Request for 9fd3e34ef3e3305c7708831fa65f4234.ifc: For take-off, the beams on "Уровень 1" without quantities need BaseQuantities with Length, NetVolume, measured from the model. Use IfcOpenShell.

First a look at what the model holds.

```python
import ifcopenshell
import ifcopenshell.util.element
import ifcopenshell.util.unit

model = ifcopenshell.open("9fd3e34ef3e3305c7708831fa65f4234.ifc")
print(model.schema)
for unit_type in ("LENGTHUNIT", "AREAUNIT", "VOLUMEUNIT"):
    print(unit_type, ifcopenshell.util.unit.calculate_unit_scale(model, unit_type))
storey = next(s for s in model.by_type("IfcBuildingStorey") if s.Name == "Уровень 1")
beams = [e for e in ifcopenshell.util.element.get_decomposition(storey) if e.is_a("IfcBeam")]
for e in sorted(beams, key=lambda e: e.id()):
    print(e.id(), e.is_a(), e.Name, list(ifcopenshell.util.element.get_psets(e, qtos_only=True)), sep=" | ")
```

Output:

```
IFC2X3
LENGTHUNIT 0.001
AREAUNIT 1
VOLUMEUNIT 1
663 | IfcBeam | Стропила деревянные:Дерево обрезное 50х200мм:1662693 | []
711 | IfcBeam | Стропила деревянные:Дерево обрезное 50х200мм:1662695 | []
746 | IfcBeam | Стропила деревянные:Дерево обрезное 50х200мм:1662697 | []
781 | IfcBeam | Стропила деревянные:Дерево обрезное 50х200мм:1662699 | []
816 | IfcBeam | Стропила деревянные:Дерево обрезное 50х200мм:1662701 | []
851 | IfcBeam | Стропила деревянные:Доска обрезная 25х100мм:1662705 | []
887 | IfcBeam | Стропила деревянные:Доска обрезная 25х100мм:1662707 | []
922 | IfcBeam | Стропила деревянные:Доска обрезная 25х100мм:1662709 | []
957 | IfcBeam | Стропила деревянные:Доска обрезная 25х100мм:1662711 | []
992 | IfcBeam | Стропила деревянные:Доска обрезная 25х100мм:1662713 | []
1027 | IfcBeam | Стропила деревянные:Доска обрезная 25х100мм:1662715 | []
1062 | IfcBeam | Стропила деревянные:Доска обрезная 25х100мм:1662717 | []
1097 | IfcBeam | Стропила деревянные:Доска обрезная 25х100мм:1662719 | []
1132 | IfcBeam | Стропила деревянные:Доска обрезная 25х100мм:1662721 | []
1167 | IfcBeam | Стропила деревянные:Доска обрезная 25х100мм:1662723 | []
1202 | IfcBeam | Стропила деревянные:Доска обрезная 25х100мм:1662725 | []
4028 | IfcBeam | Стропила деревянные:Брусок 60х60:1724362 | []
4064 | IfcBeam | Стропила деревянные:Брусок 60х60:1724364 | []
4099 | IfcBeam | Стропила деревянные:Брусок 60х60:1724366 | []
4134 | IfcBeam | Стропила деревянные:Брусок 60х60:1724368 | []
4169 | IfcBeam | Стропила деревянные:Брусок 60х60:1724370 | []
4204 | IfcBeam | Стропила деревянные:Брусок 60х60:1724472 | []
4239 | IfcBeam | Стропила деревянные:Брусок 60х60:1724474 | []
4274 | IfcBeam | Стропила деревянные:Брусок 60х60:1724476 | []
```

```python
import ifcopenshell
import ifcopenshell.api.pset
import ifcopenshell.geom
import ifcopenshell.util.element
import ifcopenshell.util.shape
import ifcopenshell.util.unit

model = ifcopenshell.open("9fd3e34ef3e3305c7708831fa65f4234.ifc")
unit_scale = ifcopenshell.util.unit.calculate_unit_scale(model)
volume_scale = ifcopenshell.util.unit.calculate_unit_scale(model, "VOLUMEUNIT")
settings = ifcopenshell.geom.settings()

storey = next(s for s in model.by_type("IfcBuildingStorey") if s.Name == "Уровень 1")
beams = [e for e in ifcopenshell.util.element.get_decomposition(storey) if e.is_a("IfcBeam")]

for e in sorted(beams, key=lambda e: e.id()):
    if ifcopenshell.util.element.get_psets(e, qtos_only=True, should_inherit=False):
        continue
    # Geometry comes back in metres, in the element's own axes.
    shape = ifcopenshell.geom.create_shape(settings, e)
    values = {
        "Length": ifcopenshell.util.shape.get_max_xyz(shape.geometry) / unit_scale,
        "NetVolume": ifcopenshell.util.shape.get_volume(shape.geometry) / volume_scale,
    }
    qto = ifcopenshell.api.pset.add_qto(model, product=e, name="BaseQuantities")
    ifcopenshell.api.pset.edit_qto(model, qto=qto, properties=values)
    print(e.id(), {k: round(v, 3) for k, v in values.items()})

model.write("9fd3e34ef3e3305c7708831fa65f4234_rev.ifc")
```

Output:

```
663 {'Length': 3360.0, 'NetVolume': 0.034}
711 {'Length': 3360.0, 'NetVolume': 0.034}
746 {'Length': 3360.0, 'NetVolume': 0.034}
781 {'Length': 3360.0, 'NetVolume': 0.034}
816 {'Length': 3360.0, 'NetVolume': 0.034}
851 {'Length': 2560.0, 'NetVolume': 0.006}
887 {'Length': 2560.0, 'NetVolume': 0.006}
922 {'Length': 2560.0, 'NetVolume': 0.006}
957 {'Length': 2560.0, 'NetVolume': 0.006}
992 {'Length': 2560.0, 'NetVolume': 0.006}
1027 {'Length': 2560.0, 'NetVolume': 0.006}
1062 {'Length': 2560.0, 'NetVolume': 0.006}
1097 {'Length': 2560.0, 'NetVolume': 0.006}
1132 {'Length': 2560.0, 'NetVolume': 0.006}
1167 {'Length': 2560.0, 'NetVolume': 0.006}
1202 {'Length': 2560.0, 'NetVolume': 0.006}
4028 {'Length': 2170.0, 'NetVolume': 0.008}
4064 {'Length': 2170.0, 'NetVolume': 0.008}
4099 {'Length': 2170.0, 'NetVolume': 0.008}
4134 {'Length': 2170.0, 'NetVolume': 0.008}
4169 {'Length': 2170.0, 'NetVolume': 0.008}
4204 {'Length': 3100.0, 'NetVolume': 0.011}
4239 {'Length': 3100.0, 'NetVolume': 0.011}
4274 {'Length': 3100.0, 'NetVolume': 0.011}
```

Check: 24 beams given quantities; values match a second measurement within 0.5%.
